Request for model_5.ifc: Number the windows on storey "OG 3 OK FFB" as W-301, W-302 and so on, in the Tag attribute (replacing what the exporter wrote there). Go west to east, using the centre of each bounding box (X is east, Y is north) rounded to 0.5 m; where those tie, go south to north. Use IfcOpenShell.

First a look at what the model holds.

```python
import ifcopenshell
import ifcopenshell.util.element
import ifcopenshell.util.placement

model = ifcopenshell.open("model_5.ifc")
print(model.schema)
storey = next(s for s in model.by_type("IfcBuildingStorey") if s.Name == "OG 3 OK FFB")
windows = [e for e in ifcopenshell.util.element.get_decomposition(storey) if e.is_a("IfcWindow")]
for e in sorted(windows, key=lambda e: e.id()):
    origin = ifcopenshell.util.placement.get_local_placement(e.ObjectPlacement)[:3, 3]
    print(e.id(), e.Tag, e.Name, origin.round(2) + 0.0, sep=" | ")
```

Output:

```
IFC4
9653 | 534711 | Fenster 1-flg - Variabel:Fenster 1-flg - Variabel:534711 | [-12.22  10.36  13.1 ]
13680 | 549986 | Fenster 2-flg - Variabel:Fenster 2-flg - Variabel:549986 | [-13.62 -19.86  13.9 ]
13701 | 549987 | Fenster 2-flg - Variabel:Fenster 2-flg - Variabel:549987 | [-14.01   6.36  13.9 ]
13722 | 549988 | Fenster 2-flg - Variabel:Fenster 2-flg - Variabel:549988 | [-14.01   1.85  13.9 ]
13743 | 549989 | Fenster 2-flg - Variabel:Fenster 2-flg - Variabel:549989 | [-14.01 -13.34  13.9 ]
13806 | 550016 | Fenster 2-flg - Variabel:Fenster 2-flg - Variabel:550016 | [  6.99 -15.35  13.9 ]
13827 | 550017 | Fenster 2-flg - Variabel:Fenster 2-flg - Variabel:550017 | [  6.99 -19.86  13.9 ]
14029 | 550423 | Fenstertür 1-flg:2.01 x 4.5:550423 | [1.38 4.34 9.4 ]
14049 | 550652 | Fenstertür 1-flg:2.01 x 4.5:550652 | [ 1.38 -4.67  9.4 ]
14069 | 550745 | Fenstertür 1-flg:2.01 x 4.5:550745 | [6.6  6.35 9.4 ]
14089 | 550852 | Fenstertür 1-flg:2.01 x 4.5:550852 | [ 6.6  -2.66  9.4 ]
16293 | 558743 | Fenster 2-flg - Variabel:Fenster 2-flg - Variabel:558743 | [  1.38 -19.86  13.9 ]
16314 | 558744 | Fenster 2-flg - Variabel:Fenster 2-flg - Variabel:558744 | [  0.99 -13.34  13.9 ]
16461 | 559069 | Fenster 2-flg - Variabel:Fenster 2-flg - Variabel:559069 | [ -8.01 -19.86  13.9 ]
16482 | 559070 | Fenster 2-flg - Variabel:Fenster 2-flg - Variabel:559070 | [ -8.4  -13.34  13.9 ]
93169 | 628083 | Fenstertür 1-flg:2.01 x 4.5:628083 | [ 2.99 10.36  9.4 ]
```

```python
import ifcopenshell
import ifcopenshell.geom
import ifcopenshell.util.element
import ifcopenshell.util.shape

model = ifcopenshell.open("model_5.ifc")
settings = ifcopenshell.geom.settings()
settings.set("use-world-coords", True)


def centre(element):
    shape = ifcopenshell.geom.create_shape(settings, element)
    return ifcopenshell.util.shape.get_bbox_centroid(shape.geometry)


storey = next(s for s in model.by_type("IfcBuildingStorey") if s.Name == "OG 3 OK FFB")
windows = [e for e in ifcopenshell.util.element.get_decomposition(storey) if e.is_a("IfcWindow")]

# Insertion points can sit at a corner or the storey origin, so sort by the geometry (in metres).
centres = {e: centre(e) for e in windows}
windows.sort(key=lambda e: (round(centres[e][0] / 0.5), centres[e][1]))

for i, e in enumerate(windows, start=1):
    number = f"W-3{i:02d}"
    e.Tag = number
    print(e.id(), number)

model.write("model_5_updated.ifc")
```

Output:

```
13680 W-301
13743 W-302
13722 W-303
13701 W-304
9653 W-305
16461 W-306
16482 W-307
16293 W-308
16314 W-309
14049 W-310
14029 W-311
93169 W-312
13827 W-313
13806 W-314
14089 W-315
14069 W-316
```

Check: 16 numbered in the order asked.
